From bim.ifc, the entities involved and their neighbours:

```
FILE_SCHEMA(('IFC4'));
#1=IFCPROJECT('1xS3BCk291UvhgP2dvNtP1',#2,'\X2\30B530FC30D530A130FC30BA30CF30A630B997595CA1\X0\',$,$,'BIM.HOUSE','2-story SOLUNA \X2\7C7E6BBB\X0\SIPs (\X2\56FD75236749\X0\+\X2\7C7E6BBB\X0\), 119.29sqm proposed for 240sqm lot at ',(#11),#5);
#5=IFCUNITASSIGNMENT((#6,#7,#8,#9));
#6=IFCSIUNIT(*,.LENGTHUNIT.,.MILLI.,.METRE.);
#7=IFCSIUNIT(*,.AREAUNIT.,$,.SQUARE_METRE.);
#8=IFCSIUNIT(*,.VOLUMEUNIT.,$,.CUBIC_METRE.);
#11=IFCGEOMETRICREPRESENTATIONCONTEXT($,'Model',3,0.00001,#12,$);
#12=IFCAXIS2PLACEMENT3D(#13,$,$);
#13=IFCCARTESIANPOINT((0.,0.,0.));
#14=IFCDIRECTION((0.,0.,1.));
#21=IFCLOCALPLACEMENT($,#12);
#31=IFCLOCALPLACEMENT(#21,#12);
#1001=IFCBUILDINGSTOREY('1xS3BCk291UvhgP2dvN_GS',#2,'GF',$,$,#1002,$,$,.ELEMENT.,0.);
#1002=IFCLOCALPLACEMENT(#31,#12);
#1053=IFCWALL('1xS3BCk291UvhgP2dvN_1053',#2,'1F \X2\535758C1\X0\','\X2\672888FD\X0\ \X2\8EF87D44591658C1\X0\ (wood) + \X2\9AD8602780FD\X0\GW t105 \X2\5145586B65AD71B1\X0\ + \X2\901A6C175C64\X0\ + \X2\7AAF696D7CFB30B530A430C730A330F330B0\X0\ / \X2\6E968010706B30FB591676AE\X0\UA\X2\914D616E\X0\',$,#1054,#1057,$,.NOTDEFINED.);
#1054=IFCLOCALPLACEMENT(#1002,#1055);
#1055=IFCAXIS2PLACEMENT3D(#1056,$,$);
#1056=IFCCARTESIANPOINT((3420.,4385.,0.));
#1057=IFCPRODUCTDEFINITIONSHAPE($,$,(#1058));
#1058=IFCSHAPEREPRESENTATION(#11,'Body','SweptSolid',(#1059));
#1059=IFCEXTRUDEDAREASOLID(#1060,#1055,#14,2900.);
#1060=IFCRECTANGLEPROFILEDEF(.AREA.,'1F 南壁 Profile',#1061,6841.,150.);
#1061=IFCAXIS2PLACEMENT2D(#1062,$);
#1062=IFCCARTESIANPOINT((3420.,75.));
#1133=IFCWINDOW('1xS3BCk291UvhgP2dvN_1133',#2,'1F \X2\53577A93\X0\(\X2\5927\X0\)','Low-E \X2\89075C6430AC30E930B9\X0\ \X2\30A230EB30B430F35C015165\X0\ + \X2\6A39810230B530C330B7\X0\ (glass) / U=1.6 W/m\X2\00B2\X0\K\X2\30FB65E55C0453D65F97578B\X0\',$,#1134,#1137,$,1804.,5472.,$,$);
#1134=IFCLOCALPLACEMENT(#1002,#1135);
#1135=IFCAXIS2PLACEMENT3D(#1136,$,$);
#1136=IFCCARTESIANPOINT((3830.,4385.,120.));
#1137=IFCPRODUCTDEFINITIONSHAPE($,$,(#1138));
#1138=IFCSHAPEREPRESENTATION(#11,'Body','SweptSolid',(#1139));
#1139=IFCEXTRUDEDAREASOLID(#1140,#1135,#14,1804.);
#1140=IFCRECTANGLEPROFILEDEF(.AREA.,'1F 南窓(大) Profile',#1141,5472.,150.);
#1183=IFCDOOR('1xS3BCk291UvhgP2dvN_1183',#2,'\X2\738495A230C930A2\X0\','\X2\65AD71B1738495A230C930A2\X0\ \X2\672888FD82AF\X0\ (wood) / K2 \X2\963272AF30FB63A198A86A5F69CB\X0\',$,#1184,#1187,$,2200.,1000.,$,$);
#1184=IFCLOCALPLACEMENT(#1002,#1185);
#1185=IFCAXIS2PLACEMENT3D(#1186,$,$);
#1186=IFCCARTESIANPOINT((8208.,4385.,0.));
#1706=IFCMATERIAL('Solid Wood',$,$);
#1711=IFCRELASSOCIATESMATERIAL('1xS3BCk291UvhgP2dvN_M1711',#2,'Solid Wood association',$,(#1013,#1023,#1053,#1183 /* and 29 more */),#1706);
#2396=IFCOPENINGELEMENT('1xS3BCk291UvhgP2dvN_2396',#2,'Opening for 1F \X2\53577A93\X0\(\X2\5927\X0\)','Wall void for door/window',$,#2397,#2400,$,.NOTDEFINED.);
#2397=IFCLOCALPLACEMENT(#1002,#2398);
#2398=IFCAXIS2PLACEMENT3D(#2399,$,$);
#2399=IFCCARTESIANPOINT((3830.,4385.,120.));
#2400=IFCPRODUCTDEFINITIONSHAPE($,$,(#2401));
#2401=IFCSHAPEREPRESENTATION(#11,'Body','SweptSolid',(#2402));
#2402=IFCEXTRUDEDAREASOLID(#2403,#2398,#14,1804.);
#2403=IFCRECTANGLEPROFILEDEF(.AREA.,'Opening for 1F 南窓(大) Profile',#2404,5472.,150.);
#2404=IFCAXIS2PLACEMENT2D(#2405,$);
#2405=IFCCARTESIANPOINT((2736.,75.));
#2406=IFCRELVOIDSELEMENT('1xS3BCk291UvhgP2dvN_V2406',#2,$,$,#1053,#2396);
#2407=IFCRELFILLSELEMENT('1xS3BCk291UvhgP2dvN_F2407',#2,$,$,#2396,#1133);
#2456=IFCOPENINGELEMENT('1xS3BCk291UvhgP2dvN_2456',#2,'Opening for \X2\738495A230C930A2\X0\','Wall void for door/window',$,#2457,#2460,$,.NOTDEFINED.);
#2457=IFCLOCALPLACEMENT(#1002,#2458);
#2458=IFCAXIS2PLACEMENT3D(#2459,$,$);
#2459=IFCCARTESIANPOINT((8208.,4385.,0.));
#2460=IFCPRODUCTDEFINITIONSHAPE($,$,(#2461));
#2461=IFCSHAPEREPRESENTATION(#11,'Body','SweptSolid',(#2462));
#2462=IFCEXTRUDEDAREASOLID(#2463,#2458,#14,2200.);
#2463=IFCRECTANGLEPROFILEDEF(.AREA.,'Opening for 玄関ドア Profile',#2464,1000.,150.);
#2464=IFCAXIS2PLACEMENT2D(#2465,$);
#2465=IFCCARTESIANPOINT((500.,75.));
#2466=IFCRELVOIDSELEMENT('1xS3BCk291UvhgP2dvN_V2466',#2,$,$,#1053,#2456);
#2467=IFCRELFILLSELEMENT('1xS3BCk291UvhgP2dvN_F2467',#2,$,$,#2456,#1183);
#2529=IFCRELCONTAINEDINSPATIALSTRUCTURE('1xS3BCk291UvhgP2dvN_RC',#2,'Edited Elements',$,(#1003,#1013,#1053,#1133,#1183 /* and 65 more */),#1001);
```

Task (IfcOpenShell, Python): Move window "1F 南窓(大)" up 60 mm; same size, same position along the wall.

```python
import numpy as np
import ifcopenshell
import ifcopenshell.api.geometry
import ifcopenshell.util.placement
import ifcopenshell.util.unit

model = ifcopenshell.open("bim.ifc")
unit_scale = ifcopenshell.util.unit.calculate_unit_scale(model)

window = model.by_guid("1xS3BCk291UvhgP2dvN_1133")
opening = window.FillsVoids[0].RelatingOpeningElement
dz = 60.0

shift = np.array([0.0, 0.0, dz])
# The window is not placed relative to its opening, so move both.
for product in (opening, window):
    matrix = ifcopenshell.util.placement.get_local_placement(product.ObjectPlacement)
    matrix[:3, 3] += shift
    ifcopenshell.api.geometry.edit_object_placement(model, product=product, matrix=matrix, is_si=False)

print(f"moved by {dz * unit_scale:+.3f} m")

model.write("bim_v2.ifc")
```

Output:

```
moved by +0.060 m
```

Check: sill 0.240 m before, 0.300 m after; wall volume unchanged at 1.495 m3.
